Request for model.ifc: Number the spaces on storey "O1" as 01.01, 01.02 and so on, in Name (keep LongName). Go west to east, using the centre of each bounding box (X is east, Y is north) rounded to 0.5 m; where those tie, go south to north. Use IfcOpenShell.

First a look at what the model holds.

```python
import ifcopenshell
import ifcopenshell.util.element
import ifcopenshell.util.placement

model = ifcopenshell.open("model.ifc")
print(model.schema)
storey = next(s for s in model.by_type("IfcBuildingStorey") if s.Name == "O1")
spaces = [e for e in ifcopenshell.util.element.get_decomposition(storey) if e.is_a("IfcSpace")]
for e in sorted(spaces, key=lambda e: e.id()):
    origin = ifcopenshell.util.placement.get_local_placement(e.ObjectPlacement)[:3, 3]
    print(e.id(), e.Name, e.LongName, origin.round(2) + 0.0, sep=" | ")
```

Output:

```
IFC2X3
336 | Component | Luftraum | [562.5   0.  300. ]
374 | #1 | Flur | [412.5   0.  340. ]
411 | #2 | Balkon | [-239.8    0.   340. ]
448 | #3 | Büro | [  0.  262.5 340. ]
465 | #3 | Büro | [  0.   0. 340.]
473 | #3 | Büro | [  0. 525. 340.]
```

```python
import ifcopenshell
import ifcopenshell.geom
import ifcopenshell.util.element
import ifcopenshell.util.shape

model = ifcopenshell.open("model.ifc")
settings = ifcopenshell.geom.settings()
settings.set("use-world-coords", True)


def centre(element):
    shape = ifcopenshell.geom.create_shape(settings, element)
    return ifcopenshell.util.shape.get_bbox_centroid(shape.geometry)


storey = next(s for s in model.by_type("IfcBuildingStorey") if s.Name == "O1")
spaces = [e for e in ifcopenshell.util.element.get_decomposition(storey) if e.is_a("IfcSpace")]

# Insertion points can sit at a corner or the storey origin, so sort by the geometry (in metres).
centres = {e: centre(e) for e in spaces}
spaces.sort(key=lambda e: (round(centres[e][0] / 0.5), centres[e][1]))

for i, e in enumerate(spaces, start=1):
    number = f"01.{i:02d}"
    e.Name = number
    print(e.id(), number)

model.write("model_updated.ifc")
```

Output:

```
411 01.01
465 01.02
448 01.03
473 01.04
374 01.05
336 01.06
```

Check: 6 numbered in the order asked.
